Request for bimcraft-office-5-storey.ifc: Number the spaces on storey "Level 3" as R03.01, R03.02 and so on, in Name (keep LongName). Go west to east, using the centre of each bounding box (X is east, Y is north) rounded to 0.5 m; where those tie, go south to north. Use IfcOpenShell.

First a look at what the model holds.

```python
import ifcopenshell
import ifcopenshell.util.element
import ifcopenshell.util.placement

model = ifcopenshell.open("bimcraft-office-5-storey.ifc")
print(model.schema)
storey = next(s for s in model.by_type("IfcBuildingStorey") if s.Name == "Level 3")
spaces = [e for e in ifcopenshell.util.element.get_decomposition(storey) if e.is_a("IfcSpace")]
for e in sorted(spaces, key=lambda e: e.id()):
    origin = ifcopenshell.util.placement.get_local_placement(e.ObjectPlacement)[:3, 3]
    print(e.id(), e.Name, e.LongName, origin.round(2) + 0.0, sep=" | ")
```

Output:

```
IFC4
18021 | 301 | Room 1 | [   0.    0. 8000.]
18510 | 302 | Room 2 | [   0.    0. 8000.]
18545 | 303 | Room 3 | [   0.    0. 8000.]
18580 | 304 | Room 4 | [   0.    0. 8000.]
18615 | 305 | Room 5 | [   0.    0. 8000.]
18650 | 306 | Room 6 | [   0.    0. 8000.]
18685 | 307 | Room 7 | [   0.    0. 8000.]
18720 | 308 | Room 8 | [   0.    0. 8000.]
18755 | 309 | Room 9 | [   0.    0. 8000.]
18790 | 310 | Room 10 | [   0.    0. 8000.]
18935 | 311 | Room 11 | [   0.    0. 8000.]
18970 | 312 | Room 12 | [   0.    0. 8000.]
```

```python
import ifcopenshell
import ifcopenshell.geom
import ifcopenshell.util.element
import ifcopenshell.util.shape

model = ifcopenshell.open("bimcraft-office-5-storey.ifc")
settings = ifcopenshell.geom.settings()
settings.set("use-world-coords", True)


def centre(element):
    shape = ifcopenshell.geom.create_shape(settings, element)
    return ifcopenshell.util.shape.get_bbox_centroid(shape.geometry)


storey = next(s for s in model.by_type("IfcBuildingStorey") if s.Name == "Level 3")
spaces = [e for e in ifcopenshell.util.element.get_decomposition(storey) if e.is_a("IfcSpace")]

# Insertion points can sit at a corner or the storey origin, so sort by the geometry (in metres).
centres = {e: centre(e) for e in spaces}
spaces.sort(key=lambda e: (round(centres[e][0] / 0.5), centres[e][1]))

for i, e in enumerate(spaces, start=1):
    number = f"R03.{i:02d}"
    e.Name = number
    print(e.id(), number)

model.write("bimcraft-office-5-storey_rev.ifc")
```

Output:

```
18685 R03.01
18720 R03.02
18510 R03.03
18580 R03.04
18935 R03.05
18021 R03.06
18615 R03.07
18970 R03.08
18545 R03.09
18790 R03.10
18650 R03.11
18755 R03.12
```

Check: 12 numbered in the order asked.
